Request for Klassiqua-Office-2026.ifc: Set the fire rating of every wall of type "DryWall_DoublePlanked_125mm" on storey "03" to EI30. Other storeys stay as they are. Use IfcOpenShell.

First a look at what the model holds.

```python
import ifcopenshell
import ifcopenshell.util.element

model = ifcopenshell.open("Klassiqua-Office-2026.ifc")
print(model.schema)
storey = next(s for s in model.by_type("IfcBuildingStorey") if s.Name == "03")
walls = [e for e in ifcopenshell.util.element.get_decomposition(storey) if e.is_a("IfcWall")]
seen = {}
for e in walls:
    element_type = ifcopenshell.util.element.get_type(e)
    key = (element_type.Name if element_type != e and element_type else None, ifcopenshell.util.element.get_pset(e, "Pset_WallCommon", "FireRating"))
    seen[key] = seen.get(key, 0) + 1
for (name, value), count in sorted(seen.items(), key=str):
    print(count, "x", name, "|", value)
```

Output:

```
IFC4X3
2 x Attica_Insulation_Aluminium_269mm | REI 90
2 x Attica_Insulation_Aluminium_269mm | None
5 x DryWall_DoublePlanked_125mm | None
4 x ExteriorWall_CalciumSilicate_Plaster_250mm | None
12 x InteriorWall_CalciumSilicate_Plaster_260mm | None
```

```python
import ifcopenshell
import ifcopenshell.api.pset
import ifcopenshell.util.element

model = ifcopenshell.open("Klassiqua-Office-2026.ifc")

storey = next(s for s in model.by_type("IfcBuildingStorey") if s.Name == "03")
walls = [e for e in ifcopenshell.util.element.get_decomposition(storey) if e.is_a("IfcWall")]

count = 0
for e in walls:
    element_type = ifcopenshell.util.element.get_type(e)
    if element_type in (None, e) or element_type.Name != "DryWall_DoublePlanked_125mm":
        continue
    # add_pset returns the element's existing set when there is one.
    pset = ifcopenshell.api.pset.add_pset(model, product=e, name="Pset_WallCommon")
    ifcopenshell.api.pset.edit_pset(model, pset=pset, properties={"FireRating": "EI30"})
    count += 1

print(count, "walls updated")

model.write("Klassiqua-Office-2026_rev.ifc")
```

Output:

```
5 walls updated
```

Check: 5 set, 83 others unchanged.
